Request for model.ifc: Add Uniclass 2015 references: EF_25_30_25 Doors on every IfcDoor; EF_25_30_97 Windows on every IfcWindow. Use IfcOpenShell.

First a look at what the model holds.

```python
import ifcopenshell

model = ifcopenshell.open("model.ifc")
print(model.schema)
print("classifications:", [c.Name for c in model.by_type("IfcClassification")])
for ifc_class in ("IfcDoor", "IfcRoof", "IfcStair", "IfcWall", "IfcWindow"):
    print(ifc_class, len(model.by_type(ifc_class)))
```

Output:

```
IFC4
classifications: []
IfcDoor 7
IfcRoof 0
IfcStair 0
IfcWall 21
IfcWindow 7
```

```python
import ifcopenshell
import ifcopenshell.api.classification

model = ifcopenshell.open("model.ifc")

system = ifcopenshell.api.classification.add_classification(model, classification="Uniclass 2015")

codes = {
    "IfcDoor": ("EF_25_30_25", "Doors"),
    "IfcWindow": ("EF_25_30_97", "Windows"),
}
for ifc_class, (code, name) in codes.items():
    products = model.by_type(ifc_class)
    ifcopenshell.api.classification.add_reference(
        model, products=products, classification=system, identification=code, name=name
    )
    print(code, len(products))

model.write("model-out.ifc")
```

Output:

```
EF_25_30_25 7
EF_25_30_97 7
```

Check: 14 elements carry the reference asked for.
